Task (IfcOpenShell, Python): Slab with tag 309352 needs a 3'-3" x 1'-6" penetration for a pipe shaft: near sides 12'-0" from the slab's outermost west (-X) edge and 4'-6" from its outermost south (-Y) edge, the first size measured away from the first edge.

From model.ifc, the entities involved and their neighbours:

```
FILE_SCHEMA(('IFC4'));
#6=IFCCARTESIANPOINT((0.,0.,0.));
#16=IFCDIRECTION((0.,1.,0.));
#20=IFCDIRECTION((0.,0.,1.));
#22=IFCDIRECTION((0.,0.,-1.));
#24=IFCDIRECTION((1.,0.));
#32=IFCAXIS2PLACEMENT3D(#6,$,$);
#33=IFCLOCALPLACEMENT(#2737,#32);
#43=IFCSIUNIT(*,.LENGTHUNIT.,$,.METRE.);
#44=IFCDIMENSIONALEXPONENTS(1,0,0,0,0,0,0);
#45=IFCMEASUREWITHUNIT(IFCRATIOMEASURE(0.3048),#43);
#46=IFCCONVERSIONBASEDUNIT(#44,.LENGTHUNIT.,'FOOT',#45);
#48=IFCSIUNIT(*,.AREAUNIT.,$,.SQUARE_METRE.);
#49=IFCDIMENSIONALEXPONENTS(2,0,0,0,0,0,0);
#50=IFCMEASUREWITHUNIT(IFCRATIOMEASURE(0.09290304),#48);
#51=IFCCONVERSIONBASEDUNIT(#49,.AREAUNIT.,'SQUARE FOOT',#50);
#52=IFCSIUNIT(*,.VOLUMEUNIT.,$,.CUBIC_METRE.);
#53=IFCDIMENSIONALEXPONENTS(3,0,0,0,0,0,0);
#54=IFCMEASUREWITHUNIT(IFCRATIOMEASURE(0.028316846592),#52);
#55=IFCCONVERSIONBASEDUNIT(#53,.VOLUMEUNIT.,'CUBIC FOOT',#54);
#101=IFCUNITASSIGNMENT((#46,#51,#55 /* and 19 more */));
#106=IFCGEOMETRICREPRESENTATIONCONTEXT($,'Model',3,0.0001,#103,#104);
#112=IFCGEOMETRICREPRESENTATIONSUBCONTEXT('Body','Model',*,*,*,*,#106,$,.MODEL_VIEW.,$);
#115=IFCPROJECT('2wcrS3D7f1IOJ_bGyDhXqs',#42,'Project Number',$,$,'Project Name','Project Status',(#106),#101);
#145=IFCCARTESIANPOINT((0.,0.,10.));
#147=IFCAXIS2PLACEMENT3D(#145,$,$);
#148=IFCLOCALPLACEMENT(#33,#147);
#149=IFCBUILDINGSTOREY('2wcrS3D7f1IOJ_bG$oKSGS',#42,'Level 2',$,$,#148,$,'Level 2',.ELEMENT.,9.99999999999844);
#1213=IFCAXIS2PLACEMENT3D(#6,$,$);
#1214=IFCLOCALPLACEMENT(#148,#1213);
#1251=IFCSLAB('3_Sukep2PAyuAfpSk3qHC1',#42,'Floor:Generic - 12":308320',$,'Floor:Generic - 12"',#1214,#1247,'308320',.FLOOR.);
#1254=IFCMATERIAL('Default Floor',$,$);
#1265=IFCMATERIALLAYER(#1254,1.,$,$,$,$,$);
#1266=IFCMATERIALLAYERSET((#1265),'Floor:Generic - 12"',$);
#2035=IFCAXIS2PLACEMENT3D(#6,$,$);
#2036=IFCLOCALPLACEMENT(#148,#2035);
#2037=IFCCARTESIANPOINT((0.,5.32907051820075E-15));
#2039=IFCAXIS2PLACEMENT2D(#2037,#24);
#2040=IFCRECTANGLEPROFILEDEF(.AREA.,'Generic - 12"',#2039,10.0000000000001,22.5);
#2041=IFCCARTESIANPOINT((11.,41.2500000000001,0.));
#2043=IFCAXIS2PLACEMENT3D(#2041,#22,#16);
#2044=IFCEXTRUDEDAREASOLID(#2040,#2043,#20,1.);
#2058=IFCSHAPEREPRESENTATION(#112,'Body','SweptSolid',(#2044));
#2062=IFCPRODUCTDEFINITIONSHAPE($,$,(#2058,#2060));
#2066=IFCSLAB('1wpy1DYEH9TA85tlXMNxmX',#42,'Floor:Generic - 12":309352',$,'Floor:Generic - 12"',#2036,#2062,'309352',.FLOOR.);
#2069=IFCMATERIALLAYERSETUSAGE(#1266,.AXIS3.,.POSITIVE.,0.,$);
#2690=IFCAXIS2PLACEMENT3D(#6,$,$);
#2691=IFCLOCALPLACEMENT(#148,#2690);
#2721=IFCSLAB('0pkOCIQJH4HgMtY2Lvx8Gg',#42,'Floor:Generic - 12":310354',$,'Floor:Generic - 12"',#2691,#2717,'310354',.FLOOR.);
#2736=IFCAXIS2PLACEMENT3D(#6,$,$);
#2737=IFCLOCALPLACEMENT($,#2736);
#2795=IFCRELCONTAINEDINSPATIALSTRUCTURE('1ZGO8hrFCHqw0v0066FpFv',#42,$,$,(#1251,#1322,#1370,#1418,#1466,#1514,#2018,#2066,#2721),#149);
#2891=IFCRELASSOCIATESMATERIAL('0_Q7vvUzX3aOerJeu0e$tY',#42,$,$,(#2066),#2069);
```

```python
import numpy as np
import ifcopenshell
import ifcopenshell.api.feature
import ifcopenshell.api.geometry
import ifcopenshell.api.root
import ifcopenshell.geom
import ifcopenshell.util.placement
import ifcopenshell.util.representation
import ifcopenshell.util.shape
import ifcopenshell.util.unit

model = ifcopenshell.open("model.ifc")
unit_scale = ifcopenshell.util.unit.calculate_unit_scale(model)
settings = ifcopenshell.geom.settings()


def volume(element):
    """Net volume in cubic metres, openings subtracted."""
    shape = ifcopenshell.geom.create_shape(settings, element)
    return ifcopenshell.util.shape.get_volume(shape.geometry)


slab = model.by_guid("1wpy1DYEH9TA85tlXMNxmX")
before = volume(slab)

# Extent in the slab's own axes, in metres. The edges named are its -X and -Y sides.
slab_shape = ifcopenshell.geom.create_shape(settings, slab)
vertices = ifcopenshell.util.shape.get_vertices(slab_shape.geometry)
x_min, y_min, bottom = vertices.min(axis=0)
top = vertices[:, 2].max()

opening = ifcopenshell.api.root.create_entity(model, ifc_class="IfcOpeningElement", name="Pipe shaft opening", predefined_type="OPENING")
context = ifcopenshell.util.representation.get_context(model, "Model", "Body", "MODEL_VIEW")
width, depth = 0.9906, 0.4572
outline = [(0.0, 0.0), (width, 0.0), (width, depth), (0.0, depth), (0.0, 0.0)]
# Overshoot both faces by 50 mm so the cut is clean.
shape = ifcopenshell.api.geometry.add_slab_representation(
    model, context=context, depth=top - bottom + 0.1, polyline=outline
)
ifcopenshell.api.geometry.assign_representation(model, product=opening, representation=shape)

matrix = ifcopenshell.util.placement.get_local_placement(slab.ObjectPlacement)
matrix[:, 3] = matrix @ np.append(np.array([x_min + 3.6576, y_min + 1.3716, bottom - 0.05]) / unit_scale, 1.0)
ifcopenshell.api.geometry.edit_object_placement(model, product=opening, matrix=matrix, is_si=False)
ifcopenshell.api.feature.add_feature(model, feature=opening, element=slab)

after = volume(slab)

print(f"slab volume {before:.3f} -> {after:.3f} m3")

model.write("model_edited.ifc")
```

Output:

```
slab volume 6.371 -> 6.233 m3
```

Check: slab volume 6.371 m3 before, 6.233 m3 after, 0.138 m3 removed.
